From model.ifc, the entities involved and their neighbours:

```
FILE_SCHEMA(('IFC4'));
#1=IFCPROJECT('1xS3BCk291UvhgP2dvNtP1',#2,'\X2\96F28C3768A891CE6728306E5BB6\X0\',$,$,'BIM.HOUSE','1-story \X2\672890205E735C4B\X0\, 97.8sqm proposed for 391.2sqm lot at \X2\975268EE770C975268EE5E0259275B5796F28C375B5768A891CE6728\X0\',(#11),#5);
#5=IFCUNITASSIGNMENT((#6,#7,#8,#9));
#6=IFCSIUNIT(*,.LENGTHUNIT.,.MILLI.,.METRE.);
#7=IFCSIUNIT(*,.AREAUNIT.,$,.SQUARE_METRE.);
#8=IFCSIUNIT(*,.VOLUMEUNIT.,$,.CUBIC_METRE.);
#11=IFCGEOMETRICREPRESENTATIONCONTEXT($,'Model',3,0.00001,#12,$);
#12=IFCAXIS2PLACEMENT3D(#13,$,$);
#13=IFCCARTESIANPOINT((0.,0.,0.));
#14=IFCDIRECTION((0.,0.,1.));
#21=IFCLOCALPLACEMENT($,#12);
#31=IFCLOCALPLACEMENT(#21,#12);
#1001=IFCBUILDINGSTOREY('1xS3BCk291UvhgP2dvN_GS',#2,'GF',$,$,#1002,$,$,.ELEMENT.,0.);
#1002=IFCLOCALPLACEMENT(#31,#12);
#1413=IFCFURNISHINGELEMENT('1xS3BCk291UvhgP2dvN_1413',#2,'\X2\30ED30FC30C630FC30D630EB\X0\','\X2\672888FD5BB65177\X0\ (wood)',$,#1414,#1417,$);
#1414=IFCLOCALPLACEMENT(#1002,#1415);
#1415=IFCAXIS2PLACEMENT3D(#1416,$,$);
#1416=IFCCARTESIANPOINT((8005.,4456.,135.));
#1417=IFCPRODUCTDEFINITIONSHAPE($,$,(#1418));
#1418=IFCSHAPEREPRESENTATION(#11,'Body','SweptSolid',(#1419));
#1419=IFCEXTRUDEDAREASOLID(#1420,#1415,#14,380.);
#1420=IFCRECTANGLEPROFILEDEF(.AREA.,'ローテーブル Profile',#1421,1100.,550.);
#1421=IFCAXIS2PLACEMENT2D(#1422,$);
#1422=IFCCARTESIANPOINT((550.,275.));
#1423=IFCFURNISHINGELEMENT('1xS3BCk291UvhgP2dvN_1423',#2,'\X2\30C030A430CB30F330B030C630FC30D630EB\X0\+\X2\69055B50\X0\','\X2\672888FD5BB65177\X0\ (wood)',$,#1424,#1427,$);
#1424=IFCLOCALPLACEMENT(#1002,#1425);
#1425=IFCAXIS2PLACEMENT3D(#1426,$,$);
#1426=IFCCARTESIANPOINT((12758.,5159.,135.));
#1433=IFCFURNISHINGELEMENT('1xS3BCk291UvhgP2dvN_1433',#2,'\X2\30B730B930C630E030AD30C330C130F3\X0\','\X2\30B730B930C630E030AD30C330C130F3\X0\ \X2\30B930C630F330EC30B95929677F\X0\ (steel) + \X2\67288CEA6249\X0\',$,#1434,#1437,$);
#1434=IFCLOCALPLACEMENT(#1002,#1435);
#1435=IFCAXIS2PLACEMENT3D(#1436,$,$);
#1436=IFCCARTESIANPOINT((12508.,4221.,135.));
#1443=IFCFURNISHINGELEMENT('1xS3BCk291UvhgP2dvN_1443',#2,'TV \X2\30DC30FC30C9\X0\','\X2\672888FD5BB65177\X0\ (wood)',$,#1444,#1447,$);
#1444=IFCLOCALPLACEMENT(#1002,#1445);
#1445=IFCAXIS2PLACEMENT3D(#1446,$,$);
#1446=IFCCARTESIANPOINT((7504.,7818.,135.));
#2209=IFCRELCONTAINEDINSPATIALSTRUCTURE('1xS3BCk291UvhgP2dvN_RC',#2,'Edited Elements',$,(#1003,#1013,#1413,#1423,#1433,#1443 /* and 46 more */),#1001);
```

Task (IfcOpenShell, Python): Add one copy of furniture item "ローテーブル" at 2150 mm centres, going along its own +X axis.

```python
import ifcopenshell
import ifcopenshell.api.geometry
import ifcopenshell.api.root
import ifcopenshell.util.element
import ifcopenshell.util.placement

model = ifcopenshell.open("model.ifc")


def reuse_history(source, copy):
    """copy_class also copies each property set's owner history, people and application; keep the originals."""
    for rel in copy.IsDefinedBy:
        if rel.is_a("IfcRelDefinesByProperties") and (history := rel.RelatingPropertyDefinition.OwnerHistory):
            rel.RelatingPropertyDefinition.OwnerHistory = source.OwnerHistory
            ifcopenshell.util.element.remove_deep2(model, history)


source = model.by_guid("1xS3BCk291UvhgP2dvN_1413")
base = ifcopenshell.util.placement.get_local_placement(source.ObjectPlacement)
step = base[:3, 0] * 2150.0

for i in range(1, 2):
    copy = ifcopenshell.api.root.copy_class(model, product=source)
    copy.Representation = ifcopenshell.util.element.copy_deep(
        model, source.Representation, exclude=["IfcGeometricRepresentationContext", "IfcRepresentationMap"]
    )
    reuse_history(source, copy)
    matrix = base.copy()
    matrix[:3, 3] += i * step
    print("added at", matrix[:3, 3].round(3) + 0.0)
    ifcopenshell.api.geometry.edit_object_placement(model, product=copy, matrix=matrix, is_si=False)

model.write("model_v2.ifc")
```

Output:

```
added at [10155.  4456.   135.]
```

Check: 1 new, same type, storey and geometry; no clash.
